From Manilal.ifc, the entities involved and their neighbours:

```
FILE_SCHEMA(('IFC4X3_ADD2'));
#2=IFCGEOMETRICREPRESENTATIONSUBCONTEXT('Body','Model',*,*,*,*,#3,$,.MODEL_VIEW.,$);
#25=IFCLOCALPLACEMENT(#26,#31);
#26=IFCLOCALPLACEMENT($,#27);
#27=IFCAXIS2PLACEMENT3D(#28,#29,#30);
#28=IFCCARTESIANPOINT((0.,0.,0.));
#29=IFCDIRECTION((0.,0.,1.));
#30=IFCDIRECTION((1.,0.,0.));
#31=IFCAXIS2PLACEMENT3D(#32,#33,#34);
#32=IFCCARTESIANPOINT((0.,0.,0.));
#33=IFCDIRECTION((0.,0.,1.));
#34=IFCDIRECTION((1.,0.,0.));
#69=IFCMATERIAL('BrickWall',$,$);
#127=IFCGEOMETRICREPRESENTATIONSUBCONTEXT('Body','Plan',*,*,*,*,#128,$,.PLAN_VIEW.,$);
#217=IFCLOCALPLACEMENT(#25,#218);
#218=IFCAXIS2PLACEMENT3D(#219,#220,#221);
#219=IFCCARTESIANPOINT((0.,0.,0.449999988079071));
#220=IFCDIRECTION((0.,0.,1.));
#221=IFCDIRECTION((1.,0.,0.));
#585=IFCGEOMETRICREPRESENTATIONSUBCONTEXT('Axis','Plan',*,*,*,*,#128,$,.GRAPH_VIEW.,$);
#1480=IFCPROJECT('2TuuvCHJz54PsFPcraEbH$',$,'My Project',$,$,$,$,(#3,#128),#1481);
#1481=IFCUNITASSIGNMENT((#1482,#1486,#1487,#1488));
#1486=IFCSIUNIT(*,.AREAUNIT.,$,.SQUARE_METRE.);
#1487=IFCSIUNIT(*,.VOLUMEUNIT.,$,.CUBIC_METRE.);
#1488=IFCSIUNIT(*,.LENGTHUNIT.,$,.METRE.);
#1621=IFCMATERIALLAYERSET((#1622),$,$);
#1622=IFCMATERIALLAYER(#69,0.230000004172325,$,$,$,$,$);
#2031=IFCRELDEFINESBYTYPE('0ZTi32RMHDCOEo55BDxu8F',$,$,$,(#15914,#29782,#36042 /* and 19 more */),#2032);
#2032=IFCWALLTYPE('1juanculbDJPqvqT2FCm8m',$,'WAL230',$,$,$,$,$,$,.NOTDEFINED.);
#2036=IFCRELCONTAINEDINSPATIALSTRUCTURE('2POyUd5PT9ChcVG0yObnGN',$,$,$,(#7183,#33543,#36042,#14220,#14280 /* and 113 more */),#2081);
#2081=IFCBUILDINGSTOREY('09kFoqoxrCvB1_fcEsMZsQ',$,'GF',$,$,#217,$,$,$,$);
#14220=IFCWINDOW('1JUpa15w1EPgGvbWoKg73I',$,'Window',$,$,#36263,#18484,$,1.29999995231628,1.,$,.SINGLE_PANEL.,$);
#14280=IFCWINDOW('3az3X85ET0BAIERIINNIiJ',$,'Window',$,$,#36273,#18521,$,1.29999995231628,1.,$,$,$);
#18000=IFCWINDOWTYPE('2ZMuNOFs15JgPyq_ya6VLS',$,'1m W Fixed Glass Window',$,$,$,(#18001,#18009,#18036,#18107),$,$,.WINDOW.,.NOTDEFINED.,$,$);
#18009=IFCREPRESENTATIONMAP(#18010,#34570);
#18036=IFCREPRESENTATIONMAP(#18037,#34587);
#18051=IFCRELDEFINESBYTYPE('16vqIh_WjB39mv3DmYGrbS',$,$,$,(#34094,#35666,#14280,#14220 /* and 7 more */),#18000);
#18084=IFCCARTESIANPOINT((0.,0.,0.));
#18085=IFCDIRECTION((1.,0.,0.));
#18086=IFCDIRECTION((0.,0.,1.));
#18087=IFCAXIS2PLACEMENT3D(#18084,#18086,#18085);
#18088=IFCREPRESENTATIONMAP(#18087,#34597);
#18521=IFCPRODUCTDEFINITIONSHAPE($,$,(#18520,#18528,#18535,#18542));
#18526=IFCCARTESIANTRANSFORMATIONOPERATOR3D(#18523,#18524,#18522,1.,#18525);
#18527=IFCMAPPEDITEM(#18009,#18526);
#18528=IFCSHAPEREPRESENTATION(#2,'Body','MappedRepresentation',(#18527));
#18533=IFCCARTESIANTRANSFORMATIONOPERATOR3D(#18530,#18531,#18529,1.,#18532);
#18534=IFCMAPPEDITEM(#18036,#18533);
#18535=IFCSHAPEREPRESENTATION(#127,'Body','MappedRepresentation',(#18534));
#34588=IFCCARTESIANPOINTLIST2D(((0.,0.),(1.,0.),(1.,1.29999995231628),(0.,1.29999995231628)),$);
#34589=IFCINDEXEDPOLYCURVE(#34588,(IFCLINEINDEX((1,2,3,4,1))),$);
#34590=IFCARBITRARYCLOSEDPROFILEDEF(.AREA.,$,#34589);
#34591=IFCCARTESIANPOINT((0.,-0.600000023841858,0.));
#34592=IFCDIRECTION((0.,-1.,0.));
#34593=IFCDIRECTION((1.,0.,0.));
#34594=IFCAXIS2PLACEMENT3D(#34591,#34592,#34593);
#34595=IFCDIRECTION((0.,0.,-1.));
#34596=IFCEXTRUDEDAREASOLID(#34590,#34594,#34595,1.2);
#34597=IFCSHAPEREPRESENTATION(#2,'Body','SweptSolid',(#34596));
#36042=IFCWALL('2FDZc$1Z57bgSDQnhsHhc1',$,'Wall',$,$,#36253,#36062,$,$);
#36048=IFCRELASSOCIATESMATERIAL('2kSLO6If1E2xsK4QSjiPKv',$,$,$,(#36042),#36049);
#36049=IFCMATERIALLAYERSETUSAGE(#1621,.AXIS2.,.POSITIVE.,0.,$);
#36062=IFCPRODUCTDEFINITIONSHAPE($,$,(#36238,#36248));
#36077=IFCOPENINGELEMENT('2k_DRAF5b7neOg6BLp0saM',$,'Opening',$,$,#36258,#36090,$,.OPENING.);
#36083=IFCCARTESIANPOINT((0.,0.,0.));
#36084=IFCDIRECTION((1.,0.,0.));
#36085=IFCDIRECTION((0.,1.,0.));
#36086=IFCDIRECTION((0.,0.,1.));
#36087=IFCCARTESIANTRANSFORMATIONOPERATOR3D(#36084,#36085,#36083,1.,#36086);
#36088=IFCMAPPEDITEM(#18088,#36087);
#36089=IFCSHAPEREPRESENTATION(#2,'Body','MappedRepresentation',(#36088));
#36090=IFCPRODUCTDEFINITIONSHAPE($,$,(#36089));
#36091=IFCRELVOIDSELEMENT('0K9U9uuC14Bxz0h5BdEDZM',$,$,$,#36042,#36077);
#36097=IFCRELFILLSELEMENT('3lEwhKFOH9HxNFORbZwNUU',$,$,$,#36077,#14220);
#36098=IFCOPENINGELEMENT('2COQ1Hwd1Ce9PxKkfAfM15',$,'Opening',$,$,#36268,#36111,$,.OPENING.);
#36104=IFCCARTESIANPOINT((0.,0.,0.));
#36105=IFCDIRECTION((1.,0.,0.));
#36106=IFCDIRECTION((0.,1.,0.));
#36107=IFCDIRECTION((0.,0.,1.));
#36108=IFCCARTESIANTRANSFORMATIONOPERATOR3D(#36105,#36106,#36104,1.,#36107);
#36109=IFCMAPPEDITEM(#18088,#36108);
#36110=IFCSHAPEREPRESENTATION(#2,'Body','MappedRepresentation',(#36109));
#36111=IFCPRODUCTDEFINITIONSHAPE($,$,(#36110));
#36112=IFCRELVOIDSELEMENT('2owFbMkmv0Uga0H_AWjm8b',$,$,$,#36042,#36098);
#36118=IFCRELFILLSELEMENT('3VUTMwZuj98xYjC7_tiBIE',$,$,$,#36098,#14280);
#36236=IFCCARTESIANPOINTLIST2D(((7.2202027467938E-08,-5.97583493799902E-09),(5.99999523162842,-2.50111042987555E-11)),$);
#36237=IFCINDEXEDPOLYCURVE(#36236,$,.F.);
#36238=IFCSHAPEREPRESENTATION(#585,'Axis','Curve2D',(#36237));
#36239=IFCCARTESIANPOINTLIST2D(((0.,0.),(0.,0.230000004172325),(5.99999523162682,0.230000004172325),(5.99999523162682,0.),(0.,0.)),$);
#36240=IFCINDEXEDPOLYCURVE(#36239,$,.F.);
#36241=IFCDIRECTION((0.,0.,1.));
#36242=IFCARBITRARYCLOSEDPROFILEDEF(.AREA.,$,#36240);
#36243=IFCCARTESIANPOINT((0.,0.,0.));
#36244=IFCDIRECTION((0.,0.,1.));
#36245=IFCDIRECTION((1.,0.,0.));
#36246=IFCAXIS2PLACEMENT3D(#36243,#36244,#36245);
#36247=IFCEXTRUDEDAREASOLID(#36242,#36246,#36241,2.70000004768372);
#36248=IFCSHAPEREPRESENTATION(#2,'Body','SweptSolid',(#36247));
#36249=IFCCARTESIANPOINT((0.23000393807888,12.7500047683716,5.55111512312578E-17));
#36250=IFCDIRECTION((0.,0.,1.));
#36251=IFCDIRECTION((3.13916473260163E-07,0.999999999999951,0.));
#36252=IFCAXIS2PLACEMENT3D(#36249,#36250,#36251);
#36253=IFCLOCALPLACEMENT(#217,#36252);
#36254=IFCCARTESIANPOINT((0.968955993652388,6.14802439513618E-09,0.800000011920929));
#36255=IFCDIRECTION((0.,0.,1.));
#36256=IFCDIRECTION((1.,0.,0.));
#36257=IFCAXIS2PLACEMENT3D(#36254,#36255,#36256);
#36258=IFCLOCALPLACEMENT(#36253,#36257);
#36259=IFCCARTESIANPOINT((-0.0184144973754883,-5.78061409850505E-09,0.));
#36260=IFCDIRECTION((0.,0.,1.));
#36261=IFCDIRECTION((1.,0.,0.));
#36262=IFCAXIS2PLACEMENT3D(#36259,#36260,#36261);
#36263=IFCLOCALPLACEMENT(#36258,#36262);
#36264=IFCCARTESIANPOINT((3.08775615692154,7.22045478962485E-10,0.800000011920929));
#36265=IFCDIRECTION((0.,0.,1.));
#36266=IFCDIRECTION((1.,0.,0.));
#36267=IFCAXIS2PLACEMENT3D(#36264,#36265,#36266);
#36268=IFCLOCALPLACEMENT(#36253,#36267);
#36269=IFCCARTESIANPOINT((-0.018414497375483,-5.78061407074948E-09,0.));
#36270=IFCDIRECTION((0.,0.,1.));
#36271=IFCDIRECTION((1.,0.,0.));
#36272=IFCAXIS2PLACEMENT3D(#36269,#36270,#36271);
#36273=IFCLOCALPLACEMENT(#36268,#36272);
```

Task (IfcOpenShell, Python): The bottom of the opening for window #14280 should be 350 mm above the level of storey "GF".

```python
import numpy as np
import ifcopenshell
import ifcopenshell.api.geometry
import ifcopenshell.geom
import ifcopenshell.util.element
import ifcopenshell.util.placement
import ifcopenshell.util.shape
import ifcopenshell.util.unit

model = ifcopenshell.open("Manilal.ifc")
unit_scale = ifcopenshell.util.unit.calculate_unit_scale(model)

window = model.by_id(14280)
opening = window.FillsVoids[0].RelatingOpeningElement
storey = ifcopenshell.util.element.get_container(window, ifc_class="IfcBuildingStorey")
level = ifcopenshell.util.placement.get_local_placement(storey.ObjectPlacement)[2, 3]

# The opening's origin need not be at the sill, so measure its lowest point.
shape = ifcopenshell.geom.create_shape(ifcopenshell.geom.settings(), opening)
bottom = ifcopenshell.util.shape.get_shape_bottom_elevation(shape, shape.geometry) / unit_scale
dz = level + 0.35 / unit_scale - bottom

shift = np.array([0.0, 0.0, dz])
# The window is placed relative to its opening, so it follows when the opening moves.
matrix = ifcopenshell.util.placement.get_local_placement(opening.ObjectPlacement)
matrix[:3, 3] += shift
ifcopenshell.api.geometry.edit_object_placement(
    model, product=opening, matrix=matrix, is_si=False, should_transform_children=True
)

print(f"moved by {dz * unit_scale:+.3f} m")

model.write("Manilal-out.ifc")
```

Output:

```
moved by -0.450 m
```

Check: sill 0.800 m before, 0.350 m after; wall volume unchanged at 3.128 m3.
